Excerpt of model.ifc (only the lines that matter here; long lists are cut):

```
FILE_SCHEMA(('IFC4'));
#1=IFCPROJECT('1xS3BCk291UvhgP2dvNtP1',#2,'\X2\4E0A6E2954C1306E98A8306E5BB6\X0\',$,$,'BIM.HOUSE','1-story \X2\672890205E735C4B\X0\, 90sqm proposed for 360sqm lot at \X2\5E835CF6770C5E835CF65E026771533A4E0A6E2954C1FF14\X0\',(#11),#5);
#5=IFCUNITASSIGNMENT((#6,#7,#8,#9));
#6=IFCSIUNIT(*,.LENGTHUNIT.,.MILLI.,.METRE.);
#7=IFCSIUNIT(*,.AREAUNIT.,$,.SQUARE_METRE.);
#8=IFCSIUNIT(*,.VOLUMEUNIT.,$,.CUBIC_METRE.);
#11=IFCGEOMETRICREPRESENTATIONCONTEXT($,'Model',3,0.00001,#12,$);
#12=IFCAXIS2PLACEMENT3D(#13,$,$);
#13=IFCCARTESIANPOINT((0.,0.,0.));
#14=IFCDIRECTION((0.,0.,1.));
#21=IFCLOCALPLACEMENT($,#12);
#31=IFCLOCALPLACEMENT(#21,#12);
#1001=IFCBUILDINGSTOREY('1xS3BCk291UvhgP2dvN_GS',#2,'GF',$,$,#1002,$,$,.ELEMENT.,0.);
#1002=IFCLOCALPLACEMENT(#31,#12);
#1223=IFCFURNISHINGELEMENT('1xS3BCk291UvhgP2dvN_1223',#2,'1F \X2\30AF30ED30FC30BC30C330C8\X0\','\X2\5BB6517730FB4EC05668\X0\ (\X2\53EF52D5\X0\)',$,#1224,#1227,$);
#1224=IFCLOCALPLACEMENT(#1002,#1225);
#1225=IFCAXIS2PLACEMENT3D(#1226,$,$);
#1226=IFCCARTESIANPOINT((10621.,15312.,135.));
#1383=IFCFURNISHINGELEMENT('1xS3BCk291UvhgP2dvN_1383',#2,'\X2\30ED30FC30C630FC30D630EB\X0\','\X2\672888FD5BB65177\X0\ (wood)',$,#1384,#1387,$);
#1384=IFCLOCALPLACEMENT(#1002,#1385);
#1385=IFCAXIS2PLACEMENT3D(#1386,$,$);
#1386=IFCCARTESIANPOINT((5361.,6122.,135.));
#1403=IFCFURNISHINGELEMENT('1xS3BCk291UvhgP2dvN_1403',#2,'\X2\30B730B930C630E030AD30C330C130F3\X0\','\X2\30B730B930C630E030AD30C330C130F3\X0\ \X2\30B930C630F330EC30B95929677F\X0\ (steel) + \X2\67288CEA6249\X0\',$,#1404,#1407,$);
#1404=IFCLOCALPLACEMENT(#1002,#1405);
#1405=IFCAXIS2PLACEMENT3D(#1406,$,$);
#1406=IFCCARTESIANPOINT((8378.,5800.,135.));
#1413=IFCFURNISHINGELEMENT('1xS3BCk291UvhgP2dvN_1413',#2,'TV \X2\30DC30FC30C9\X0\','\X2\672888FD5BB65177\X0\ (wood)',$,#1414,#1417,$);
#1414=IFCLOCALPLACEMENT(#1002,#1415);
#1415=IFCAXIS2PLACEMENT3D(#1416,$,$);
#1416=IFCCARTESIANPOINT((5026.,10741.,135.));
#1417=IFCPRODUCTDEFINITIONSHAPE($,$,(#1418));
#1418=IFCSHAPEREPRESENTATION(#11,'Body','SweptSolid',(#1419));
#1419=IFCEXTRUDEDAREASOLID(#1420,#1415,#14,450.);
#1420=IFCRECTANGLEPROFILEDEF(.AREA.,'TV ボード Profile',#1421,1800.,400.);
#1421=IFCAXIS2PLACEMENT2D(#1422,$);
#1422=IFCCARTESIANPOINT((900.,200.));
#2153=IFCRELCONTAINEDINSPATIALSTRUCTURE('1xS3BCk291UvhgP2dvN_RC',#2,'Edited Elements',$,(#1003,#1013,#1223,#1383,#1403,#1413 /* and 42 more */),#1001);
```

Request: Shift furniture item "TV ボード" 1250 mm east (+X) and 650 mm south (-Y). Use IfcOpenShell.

```python
import ifcopenshell
import ifcopenshell.api.geometry
import ifcopenshell.util.placement
import ifcopenshell.util.unit

model = ifcopenshell.open("model.ifc")
unit_scale = ifcopenshell.util.unit.calculate_unit_scale(model)

item = model.by_guid("1xS3BCk291UvhgP2dvN_1413")
matrix = ifcopenshell.util.placement.get_local_placement(item.ObjectPlacement)
matrix[0, 3] += 1.25 / unit_scale
matrix[1, 3] -= 0.65 / unit_scale
ifcopenshell.api.geometry.edit_object_placement(model, product=item, matrix=matrix, is_si=False)

print(ifcopenshell.util.placement.get_local_placement(item.ObjectPlacement).round(3) + 0.0)

model.write("model-out.ifc")
```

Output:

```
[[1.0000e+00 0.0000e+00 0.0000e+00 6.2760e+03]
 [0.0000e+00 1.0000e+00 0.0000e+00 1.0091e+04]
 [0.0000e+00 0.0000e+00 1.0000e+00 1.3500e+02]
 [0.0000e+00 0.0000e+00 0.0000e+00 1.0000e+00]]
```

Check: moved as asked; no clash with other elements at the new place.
